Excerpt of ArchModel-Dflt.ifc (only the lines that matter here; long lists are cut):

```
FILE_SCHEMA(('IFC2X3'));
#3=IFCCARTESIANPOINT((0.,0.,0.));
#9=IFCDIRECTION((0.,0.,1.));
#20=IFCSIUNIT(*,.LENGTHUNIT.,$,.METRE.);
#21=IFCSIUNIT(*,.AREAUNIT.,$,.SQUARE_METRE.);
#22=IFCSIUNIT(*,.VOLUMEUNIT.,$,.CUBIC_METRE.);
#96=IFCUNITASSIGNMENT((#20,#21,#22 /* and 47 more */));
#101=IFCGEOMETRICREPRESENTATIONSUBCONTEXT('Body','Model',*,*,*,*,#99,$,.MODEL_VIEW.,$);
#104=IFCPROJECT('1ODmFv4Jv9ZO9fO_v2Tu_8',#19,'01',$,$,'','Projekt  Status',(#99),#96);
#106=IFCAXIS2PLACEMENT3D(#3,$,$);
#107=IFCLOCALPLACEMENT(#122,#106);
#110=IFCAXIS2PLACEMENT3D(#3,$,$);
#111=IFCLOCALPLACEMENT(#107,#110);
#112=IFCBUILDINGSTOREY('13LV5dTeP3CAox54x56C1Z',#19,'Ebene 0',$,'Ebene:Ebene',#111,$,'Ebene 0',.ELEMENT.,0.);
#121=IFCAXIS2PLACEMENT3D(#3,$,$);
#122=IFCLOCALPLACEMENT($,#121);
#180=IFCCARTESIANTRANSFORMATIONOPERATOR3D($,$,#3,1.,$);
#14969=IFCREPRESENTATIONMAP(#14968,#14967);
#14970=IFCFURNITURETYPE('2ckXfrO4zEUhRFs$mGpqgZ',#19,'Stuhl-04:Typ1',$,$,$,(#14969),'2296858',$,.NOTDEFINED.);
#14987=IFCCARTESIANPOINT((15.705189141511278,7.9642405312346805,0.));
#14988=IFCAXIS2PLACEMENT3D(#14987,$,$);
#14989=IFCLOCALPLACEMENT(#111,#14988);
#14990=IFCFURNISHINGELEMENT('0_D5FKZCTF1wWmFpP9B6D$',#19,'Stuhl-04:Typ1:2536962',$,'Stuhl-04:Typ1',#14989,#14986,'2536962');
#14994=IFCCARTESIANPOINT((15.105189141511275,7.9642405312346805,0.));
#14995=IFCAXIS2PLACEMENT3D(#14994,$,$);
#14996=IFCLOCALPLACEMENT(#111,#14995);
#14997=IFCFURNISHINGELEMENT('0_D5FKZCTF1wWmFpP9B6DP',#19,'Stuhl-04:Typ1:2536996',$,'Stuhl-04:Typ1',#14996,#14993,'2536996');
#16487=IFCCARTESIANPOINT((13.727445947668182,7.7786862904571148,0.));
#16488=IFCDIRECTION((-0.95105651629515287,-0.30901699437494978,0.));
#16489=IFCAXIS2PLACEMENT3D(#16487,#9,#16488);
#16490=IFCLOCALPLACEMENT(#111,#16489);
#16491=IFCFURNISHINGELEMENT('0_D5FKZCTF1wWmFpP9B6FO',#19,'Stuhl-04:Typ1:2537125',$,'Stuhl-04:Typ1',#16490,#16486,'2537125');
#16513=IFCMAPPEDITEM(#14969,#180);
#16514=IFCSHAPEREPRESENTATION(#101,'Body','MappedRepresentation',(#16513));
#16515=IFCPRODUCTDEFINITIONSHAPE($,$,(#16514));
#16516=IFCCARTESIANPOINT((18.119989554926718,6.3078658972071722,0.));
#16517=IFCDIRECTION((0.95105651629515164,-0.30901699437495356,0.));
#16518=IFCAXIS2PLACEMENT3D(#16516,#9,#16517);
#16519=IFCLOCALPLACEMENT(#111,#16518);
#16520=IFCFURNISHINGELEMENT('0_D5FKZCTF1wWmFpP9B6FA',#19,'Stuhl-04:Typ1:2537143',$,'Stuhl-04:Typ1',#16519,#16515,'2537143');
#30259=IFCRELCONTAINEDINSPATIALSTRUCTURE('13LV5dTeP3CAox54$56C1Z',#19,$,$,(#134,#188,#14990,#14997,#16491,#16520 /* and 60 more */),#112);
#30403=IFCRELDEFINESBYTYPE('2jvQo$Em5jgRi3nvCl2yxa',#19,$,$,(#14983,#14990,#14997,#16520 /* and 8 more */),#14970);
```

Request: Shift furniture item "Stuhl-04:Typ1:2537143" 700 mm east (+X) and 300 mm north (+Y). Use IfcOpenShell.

```python
import ifcopenshell
import ifcopenshell.api.geometry
import ifcopenshell.util.placement
import ifcopenshell.util.unit

model = ifcopenshell.open("ArchModel-Dflt.ifc")
unit_scale = ifcopenshell.util.unit.calculate_unit_scale(model)

item = model.by_guid("0_D5FKZCTF1wWmFpP9B6FA")
matrix = ifcopenshell.util.placement.get_local_placement(item.ObjectPlacement)
matrix[0, 3] += 0.7 / unit_scale
matrix[1, 3] += 0.3 / unit_scale
ifcopenshell.api.geometry.edit_object_placement(model, product=item, matrix=matrix, is_si=False)

print(ifcopenshell.util.placement.get_local_placement(item.ObjectPlacement).round(3) + 0.0)

model.write("ArchModel-Dflt_v2.ifc")
```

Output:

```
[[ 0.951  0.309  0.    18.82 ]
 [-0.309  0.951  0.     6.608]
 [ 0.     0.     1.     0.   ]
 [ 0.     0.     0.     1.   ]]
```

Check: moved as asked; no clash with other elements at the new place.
